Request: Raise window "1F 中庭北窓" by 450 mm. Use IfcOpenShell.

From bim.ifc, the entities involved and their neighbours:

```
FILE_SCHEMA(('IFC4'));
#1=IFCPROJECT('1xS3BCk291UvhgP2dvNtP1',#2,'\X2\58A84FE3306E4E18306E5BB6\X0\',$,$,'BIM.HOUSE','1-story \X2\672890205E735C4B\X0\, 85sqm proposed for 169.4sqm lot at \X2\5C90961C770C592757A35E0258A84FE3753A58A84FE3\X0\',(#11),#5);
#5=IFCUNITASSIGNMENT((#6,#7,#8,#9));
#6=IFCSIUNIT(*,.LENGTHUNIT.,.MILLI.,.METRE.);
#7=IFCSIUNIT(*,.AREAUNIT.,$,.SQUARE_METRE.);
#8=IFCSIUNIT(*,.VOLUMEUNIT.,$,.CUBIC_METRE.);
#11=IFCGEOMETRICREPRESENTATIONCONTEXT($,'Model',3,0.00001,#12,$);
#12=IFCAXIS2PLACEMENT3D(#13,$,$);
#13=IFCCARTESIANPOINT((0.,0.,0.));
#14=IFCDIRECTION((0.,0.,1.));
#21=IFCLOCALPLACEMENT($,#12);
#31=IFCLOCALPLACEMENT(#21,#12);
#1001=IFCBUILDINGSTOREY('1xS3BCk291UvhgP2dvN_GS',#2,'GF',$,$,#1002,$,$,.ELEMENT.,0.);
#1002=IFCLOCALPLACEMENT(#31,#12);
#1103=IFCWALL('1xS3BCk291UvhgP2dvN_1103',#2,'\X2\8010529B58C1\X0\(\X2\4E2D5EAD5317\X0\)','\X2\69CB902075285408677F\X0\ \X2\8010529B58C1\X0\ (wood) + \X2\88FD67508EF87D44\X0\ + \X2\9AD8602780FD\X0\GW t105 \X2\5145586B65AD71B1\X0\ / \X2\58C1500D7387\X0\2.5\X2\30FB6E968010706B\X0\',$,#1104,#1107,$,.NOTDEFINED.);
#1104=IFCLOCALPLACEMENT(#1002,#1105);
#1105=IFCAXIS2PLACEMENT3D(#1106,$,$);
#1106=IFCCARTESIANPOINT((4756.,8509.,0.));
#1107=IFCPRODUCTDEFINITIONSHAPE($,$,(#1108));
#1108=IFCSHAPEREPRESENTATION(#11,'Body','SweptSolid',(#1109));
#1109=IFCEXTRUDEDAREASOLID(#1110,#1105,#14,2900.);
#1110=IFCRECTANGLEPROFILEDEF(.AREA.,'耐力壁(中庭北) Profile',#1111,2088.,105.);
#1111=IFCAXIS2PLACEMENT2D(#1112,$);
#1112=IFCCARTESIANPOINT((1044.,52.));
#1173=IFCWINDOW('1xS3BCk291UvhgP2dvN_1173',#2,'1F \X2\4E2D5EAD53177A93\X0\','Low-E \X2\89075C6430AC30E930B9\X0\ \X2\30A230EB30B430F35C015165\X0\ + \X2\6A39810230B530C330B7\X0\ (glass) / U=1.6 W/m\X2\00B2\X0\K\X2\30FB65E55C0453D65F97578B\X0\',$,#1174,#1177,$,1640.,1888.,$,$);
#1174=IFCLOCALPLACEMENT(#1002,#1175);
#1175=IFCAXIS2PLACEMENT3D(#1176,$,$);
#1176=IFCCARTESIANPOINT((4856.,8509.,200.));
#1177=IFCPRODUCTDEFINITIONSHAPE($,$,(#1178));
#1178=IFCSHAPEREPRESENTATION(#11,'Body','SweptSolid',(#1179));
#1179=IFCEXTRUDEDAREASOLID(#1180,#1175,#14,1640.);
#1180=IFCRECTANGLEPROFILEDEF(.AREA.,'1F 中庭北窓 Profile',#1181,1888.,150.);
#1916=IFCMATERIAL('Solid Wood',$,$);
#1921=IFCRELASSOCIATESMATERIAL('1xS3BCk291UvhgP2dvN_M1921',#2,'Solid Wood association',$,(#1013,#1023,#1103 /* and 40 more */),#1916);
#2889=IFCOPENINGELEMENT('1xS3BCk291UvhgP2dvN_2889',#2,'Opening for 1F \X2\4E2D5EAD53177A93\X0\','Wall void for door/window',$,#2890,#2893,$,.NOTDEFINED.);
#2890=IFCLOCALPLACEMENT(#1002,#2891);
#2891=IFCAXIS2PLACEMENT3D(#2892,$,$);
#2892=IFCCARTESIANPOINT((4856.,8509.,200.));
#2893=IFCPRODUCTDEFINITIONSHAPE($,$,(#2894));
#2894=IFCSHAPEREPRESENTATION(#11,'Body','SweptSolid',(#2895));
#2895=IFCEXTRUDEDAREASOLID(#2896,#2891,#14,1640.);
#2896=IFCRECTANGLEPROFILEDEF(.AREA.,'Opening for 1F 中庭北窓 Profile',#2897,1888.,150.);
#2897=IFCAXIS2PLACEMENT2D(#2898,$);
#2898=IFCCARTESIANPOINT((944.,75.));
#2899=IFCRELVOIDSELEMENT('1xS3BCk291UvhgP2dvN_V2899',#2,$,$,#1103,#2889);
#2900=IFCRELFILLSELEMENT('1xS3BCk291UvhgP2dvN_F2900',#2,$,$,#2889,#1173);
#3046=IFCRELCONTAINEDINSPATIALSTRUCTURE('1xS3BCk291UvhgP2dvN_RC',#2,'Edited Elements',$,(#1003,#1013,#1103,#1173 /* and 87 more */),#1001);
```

```python
import numpy as np
import ifcopenshell
import ifcopenshell.api.geometry
import ifcopenshell.util.placement
import ifcopenshell.util.unit

model = ifcopenshell.open("bim.ifc")
unit_scale = ifcopenshell.util.unit.calculate_unit_scale(model)

window = model.by_guid("1xS3BCk291UvhgP2dvN_1173")
opening = window.FillsVoids[0].RelatingOpeningElement
dz = 0.45 / unit_scale

shift = np.array([0.0, 0.0, dz])
# The window is not placed relative to its opening, so move both.
for product in (opening, window):
    matrix = ifcopenshell.util.placement.get_local_placement(product.ObjectPlacement)
    matrix[:3, 3] += shift
    ifcopenshell.api.geometry.edit_object_placement(model, product=product, matrix=matrix, is_si=False)

print(f"moved by {dz * unit_scale:+.3f} m")

model.write("bim_edited.ifc")
```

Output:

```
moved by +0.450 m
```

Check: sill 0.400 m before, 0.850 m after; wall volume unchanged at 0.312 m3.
